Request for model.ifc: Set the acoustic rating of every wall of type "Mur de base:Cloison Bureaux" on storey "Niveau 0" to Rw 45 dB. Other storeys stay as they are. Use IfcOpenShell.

First a look at what the model holds.

```python
import ifcopenshell
import ifcopenshell.util.element

model = ifcopenshell.open("model.ifc")
print(model.schema)
storey = next(s for s in model.by_type("IfcBuildingStorey") if s.Name == "Niveau 0")
walls = [e for e in ifcopenshell.util.element.get_decomposition(storey) if e.is_a("IfcWall")]
seen = {}
for e in walls:
    element_type = ifcopenshell.util.element.get_type(e)
    key = (element_type.Name if element_type != e and element_type else None, ifcopenshell.util.element.get_pset(e, "Pset_WallCommon", "AcousticRating"))
    seen[key] = seen.get(key, 0) + 1
for (name, value), count in sorted(seen.items(), key=str):
    print(count, "x", name, "|", value)
```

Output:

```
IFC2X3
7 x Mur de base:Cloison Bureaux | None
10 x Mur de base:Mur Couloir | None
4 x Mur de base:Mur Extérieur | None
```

```python
import ifcopenshell
import ifcopenshell.api.pset
import ifcopenshell.util.element

model = ifcopenshell.open("model.ifc")

storey = next(s for s in model.by_type("IfcBuildingStorey") if s.Name == "Niveau 0")
walls = [e for e in ifcopenshell.util.element.get_decomposition(storey) if e.is_a("IfcWall")]

count = 0
for e in walls:
    element_type = ifcopenshell.util.element.get_type(e)
    if element_type in (None, e) or element_type.Name != "Mur de base:Cloison Bureaux":
        continue
    # add_pset returns the element's existing set when there is one.
    pset = ifcopenshell.api.pset.add_pset(model, product=e, name="Pset_WallCommon")
    ifcopenshell.api.pset.edit_pset(model, pset=pset, properties={"AcousticRating": "Rw 45 dB"})
    count += 1

print(count, "walls updated")

model.write("model_rev.ifc")
```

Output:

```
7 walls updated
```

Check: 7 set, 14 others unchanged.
